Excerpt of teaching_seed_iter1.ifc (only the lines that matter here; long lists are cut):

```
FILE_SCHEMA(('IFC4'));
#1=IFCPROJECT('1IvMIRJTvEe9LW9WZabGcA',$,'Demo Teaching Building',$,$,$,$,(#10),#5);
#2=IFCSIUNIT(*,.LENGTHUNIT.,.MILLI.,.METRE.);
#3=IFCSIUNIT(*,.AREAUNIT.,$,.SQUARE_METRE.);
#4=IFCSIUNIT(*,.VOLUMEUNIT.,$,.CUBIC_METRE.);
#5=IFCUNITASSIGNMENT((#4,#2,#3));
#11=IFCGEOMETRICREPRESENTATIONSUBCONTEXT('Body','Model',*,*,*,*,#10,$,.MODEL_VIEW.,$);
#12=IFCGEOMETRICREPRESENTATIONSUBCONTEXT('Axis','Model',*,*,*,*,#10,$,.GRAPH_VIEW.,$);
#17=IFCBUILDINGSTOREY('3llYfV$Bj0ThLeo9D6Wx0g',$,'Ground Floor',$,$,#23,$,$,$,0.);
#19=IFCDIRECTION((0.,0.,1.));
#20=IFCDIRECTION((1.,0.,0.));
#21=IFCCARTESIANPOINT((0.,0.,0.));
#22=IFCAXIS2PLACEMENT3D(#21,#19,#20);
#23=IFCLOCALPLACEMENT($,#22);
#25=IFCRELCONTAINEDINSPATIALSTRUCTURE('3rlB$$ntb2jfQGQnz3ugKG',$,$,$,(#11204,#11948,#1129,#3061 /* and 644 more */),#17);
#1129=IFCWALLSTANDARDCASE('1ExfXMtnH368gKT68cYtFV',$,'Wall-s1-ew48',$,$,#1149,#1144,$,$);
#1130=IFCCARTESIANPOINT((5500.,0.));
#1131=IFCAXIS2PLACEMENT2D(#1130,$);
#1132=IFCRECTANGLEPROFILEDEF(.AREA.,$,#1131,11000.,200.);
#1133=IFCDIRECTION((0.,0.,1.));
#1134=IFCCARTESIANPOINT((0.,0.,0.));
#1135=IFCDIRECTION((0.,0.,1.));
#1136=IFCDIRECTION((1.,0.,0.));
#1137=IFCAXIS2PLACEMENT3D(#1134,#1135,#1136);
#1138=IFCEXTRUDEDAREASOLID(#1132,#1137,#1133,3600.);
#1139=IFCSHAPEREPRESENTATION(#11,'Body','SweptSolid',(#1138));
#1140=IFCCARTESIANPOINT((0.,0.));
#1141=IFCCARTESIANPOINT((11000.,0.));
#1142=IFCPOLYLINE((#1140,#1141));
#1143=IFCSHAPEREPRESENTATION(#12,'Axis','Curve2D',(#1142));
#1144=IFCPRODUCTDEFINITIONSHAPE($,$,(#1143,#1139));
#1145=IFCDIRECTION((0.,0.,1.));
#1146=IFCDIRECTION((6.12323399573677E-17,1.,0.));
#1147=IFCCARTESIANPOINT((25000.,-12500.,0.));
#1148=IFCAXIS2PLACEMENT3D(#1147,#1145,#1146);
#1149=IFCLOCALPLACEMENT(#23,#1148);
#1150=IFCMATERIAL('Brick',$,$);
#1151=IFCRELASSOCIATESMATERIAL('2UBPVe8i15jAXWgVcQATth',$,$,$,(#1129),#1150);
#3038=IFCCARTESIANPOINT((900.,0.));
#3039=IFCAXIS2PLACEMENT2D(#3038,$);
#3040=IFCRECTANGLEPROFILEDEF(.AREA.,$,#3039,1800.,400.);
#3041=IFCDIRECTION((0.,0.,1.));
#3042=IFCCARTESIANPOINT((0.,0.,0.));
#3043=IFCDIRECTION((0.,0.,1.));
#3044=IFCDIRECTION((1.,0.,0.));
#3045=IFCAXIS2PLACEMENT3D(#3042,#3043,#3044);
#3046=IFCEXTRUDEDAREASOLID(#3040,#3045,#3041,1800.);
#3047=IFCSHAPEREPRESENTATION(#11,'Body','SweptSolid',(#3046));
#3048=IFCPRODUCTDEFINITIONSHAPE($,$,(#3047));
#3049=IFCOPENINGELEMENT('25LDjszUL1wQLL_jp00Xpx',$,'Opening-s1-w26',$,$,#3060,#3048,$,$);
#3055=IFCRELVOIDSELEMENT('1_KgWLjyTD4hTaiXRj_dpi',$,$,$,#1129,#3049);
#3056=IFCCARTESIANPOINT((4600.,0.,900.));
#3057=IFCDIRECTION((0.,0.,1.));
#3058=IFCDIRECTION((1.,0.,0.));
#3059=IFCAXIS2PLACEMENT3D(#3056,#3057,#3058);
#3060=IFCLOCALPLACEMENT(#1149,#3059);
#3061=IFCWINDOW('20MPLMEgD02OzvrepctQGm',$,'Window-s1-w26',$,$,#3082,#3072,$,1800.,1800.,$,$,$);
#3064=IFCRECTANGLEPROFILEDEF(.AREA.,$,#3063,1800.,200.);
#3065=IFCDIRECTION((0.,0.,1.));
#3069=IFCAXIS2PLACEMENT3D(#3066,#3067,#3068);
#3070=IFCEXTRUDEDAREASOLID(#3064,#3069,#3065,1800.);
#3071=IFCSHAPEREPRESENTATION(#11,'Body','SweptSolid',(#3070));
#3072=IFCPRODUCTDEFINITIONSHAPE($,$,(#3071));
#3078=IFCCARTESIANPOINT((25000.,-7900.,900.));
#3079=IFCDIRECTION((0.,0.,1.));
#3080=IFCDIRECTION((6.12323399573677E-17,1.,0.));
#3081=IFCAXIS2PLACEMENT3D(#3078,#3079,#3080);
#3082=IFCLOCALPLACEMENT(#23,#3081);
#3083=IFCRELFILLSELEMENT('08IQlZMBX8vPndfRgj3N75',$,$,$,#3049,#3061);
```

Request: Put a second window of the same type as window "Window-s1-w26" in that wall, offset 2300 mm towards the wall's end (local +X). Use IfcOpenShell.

```python
import ifcopenshell
import ifcopenshell.api.feature
import ifcopenshell.api.geometry
import ifcopenshell.api.root
import ifcopenshell.geom
import ifcopenshell.util.element
import ifcopenshell.util.placement
import ifcopenshell.util.shape
import ifcopenshell.util.unit

model = ifcopenshell.open("teaching_seed_iter1.ifc")
unit_scale = ifcopenshell.util.unit.calculate_unit_scale(model)
settings = ifcopenshell.geom.settings()


def volume(element):
    """Net volume in cubic metres, openings subtracted."""
    shape = ifcopenshell.geom.create_shape(settings, element)
    return ifcopenshell.util.shape.get_volume(shape.geometry)


window = model.by_guid("20MPLMEgD02OzvrepctQGm")
opening = window.FillsVoids[0].RelatingOpeningElement
wall = opening.VoidsElements[0].RelatingBuildingElement
before = volume(wall)
shift = ifcopenshell.util.placement.get_local_placement(wall.ObjectPlacement)[:3, 0] * 2.3 / unit_scale

# copy_class copies the void relationship, type, container and properties, but no geometry.
new_opening = ifcopenshell.api.root.copy_class(model, product=opening)
new_opening.Representation = ifcopenshell.util.element.copy_deep(
    model, opening.Representation, exclude=["IfcGeometricRepresentationContext", "IfcRepresentationMap"]
)
new_window = ifcopenshell.api.root.copy_class(model, product=window)
new_window.Representation = ifcopenshell.util.element.copy_deep(
    model, window.Representation, exclude=["IfcGeometricRepresentationContext", "IfcRepresentationMap"]
)
ifcopenshell.api.feature.add_filling(model, opening=new_opening, element=new_window)

for old, new in ((opening, new_opening), (window, new_window)):
    matrix = ifcopenshell.util.placement.get_local_placement(old.ObjectPlacement)
    matrix[:3, 3] += shift
    ifcopenshell.api.geometry.edit_object_placement(model, product=new, matrix=matrix, is_si=False)

after = volume(wall)

print(f"wall volume {before:.3f} -> {after:.3f} m3")

model.write("teaching_seed_iter1-out.ifc")
```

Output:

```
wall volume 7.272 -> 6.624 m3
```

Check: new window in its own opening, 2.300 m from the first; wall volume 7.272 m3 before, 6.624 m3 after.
